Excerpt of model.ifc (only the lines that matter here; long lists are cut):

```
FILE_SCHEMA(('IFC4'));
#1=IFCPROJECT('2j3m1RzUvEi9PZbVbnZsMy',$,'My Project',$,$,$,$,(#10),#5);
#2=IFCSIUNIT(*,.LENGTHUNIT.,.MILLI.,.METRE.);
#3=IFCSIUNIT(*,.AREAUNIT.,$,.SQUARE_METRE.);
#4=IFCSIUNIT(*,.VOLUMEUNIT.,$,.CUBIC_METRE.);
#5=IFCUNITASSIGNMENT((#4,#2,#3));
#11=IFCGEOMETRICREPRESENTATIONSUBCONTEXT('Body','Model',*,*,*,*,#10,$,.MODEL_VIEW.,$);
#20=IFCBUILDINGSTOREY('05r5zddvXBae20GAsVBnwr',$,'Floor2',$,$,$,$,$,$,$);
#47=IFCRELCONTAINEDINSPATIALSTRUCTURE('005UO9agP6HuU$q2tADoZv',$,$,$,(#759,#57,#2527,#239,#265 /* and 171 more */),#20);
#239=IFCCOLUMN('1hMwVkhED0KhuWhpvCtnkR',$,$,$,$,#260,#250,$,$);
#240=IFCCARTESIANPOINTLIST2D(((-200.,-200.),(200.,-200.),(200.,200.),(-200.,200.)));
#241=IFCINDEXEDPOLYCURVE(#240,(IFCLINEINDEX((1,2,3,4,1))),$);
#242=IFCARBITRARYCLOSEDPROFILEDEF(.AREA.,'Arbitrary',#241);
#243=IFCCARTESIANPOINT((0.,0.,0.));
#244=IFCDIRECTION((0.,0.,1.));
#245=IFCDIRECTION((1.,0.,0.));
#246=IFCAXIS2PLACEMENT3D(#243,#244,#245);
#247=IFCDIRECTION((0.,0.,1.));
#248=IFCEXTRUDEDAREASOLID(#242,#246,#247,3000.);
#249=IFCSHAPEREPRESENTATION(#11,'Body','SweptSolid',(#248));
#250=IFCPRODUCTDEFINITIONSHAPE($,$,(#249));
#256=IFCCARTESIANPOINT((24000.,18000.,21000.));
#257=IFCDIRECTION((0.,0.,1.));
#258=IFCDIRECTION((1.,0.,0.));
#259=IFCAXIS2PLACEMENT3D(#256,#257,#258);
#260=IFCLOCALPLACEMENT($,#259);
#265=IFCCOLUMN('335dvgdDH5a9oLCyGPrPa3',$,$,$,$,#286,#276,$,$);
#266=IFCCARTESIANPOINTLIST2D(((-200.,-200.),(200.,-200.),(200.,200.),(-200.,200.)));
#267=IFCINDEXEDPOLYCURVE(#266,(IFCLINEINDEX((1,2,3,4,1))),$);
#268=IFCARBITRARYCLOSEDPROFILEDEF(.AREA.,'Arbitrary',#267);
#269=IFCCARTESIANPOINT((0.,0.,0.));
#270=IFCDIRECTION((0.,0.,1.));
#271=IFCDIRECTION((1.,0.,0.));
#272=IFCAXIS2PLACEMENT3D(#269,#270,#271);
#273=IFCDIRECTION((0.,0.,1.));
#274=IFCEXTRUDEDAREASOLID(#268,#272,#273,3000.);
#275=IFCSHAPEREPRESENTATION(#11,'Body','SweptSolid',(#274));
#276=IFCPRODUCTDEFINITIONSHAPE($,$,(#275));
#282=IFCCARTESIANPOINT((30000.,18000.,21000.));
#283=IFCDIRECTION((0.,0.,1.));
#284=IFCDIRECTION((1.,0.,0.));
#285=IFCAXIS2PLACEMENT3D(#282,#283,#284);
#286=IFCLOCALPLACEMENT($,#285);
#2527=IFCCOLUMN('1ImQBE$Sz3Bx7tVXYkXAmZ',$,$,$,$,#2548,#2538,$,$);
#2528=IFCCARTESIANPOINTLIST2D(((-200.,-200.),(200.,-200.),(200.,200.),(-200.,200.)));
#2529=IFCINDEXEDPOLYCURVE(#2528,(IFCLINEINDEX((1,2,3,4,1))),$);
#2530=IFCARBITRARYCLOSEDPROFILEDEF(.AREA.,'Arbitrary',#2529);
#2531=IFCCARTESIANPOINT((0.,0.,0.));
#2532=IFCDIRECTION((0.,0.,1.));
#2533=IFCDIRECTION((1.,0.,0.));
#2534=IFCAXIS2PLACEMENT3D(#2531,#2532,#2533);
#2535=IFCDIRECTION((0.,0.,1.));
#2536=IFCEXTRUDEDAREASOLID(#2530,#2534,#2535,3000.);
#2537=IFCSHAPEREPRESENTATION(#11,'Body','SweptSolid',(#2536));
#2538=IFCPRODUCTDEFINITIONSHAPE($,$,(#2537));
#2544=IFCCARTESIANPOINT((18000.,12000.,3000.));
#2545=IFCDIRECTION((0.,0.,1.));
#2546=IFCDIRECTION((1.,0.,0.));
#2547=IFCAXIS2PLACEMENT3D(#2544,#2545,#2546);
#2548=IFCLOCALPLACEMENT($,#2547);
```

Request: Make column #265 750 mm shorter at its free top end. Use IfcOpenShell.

```python
import ifcopenshell
import ifcopenshell.util.representation
import ifcopenshell.util.unit

model = ifcopenshell.open("model.ifc")
unit_scale = ifcopenshell.util.unit.calculate_unit_scale(model)

member = model.by_guid("335dvgdDH5a9oLCyGPrPa3")
change = -0.75 / unit_scale

# The extrusion runs towards the end named, so only its depth changes.
body = ifcopenshell.util.representation.get_representation(member, "Model", "Body")
solid = body.Items[0]
old_length = solid.Depth
solid.Depth += change

print(f"length {old_length:g} -> {solid.Depth:g}")

model.write("model_updated.ifc")
```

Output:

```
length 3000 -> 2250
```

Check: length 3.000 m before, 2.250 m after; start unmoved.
